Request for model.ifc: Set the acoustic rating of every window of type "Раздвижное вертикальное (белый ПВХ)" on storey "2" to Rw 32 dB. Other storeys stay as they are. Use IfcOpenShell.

First a look at what the model holds.

```python
import ifcopenshell
import ifcopenshell.util.element

model = ifcopenshell.open("model.ifc")
print(model.schema)
storey = next(s for s in model.by_type("IfcBuildingStorey") if s.Name == "2")
windows = [e for e in ifcopenshell.util.element.get_decomposition(storey) if e.is_a("IfcWindow")]
seen = {}
for e in windows:
    element_type = ifcopenshell.util.element.get_type(e)
    key = (element_type.Name if element_type != e and element_type else None, ifcopenshell.util.element.get_pset(e, "Pset_WindowCommon", "AcousticRating"))
    seen[key] = seen.get(key, 0) + 1
for (name, value), count in sorted(seen.items(), key=str):
    print(count, "x", name, "|", value)
```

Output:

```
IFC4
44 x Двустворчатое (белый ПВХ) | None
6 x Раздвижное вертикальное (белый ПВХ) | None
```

```python
import ifcopenshell
import ifcopenshell.api.pset
import ifcopenshell.util.element

model = ifcopenshell.open("model.ifc")

storey = next(s for s in model.by_type("IfcBuildingStorey") if s.Name == "2")
windows = [e for e in ifcopenshell.util.element.get_decomposition(storey) if e.is_a("IfcWindow")]

count = 0
for e in windows:
    element_type = ifcopenshell.util.element.get_type(e)
    if element_type in (None, e) or element_type.Name != "Раздвижное вертикальное (белый ПВХ)":
        continue
    # add_pset returns the element's existing set when there is one.
    pset = ifcopenshell.api.pset.add_pset(model, product=e, name="Pset_WindowCommon")
    ifcopenshell.api.pset.edit_pset(model, pset=pset, properties={"AcousticRating": "Rw 32 dB"})
    count += 1

print(count, "windows updated")

model.write("model_rev.ifc")
```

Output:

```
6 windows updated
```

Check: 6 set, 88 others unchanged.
